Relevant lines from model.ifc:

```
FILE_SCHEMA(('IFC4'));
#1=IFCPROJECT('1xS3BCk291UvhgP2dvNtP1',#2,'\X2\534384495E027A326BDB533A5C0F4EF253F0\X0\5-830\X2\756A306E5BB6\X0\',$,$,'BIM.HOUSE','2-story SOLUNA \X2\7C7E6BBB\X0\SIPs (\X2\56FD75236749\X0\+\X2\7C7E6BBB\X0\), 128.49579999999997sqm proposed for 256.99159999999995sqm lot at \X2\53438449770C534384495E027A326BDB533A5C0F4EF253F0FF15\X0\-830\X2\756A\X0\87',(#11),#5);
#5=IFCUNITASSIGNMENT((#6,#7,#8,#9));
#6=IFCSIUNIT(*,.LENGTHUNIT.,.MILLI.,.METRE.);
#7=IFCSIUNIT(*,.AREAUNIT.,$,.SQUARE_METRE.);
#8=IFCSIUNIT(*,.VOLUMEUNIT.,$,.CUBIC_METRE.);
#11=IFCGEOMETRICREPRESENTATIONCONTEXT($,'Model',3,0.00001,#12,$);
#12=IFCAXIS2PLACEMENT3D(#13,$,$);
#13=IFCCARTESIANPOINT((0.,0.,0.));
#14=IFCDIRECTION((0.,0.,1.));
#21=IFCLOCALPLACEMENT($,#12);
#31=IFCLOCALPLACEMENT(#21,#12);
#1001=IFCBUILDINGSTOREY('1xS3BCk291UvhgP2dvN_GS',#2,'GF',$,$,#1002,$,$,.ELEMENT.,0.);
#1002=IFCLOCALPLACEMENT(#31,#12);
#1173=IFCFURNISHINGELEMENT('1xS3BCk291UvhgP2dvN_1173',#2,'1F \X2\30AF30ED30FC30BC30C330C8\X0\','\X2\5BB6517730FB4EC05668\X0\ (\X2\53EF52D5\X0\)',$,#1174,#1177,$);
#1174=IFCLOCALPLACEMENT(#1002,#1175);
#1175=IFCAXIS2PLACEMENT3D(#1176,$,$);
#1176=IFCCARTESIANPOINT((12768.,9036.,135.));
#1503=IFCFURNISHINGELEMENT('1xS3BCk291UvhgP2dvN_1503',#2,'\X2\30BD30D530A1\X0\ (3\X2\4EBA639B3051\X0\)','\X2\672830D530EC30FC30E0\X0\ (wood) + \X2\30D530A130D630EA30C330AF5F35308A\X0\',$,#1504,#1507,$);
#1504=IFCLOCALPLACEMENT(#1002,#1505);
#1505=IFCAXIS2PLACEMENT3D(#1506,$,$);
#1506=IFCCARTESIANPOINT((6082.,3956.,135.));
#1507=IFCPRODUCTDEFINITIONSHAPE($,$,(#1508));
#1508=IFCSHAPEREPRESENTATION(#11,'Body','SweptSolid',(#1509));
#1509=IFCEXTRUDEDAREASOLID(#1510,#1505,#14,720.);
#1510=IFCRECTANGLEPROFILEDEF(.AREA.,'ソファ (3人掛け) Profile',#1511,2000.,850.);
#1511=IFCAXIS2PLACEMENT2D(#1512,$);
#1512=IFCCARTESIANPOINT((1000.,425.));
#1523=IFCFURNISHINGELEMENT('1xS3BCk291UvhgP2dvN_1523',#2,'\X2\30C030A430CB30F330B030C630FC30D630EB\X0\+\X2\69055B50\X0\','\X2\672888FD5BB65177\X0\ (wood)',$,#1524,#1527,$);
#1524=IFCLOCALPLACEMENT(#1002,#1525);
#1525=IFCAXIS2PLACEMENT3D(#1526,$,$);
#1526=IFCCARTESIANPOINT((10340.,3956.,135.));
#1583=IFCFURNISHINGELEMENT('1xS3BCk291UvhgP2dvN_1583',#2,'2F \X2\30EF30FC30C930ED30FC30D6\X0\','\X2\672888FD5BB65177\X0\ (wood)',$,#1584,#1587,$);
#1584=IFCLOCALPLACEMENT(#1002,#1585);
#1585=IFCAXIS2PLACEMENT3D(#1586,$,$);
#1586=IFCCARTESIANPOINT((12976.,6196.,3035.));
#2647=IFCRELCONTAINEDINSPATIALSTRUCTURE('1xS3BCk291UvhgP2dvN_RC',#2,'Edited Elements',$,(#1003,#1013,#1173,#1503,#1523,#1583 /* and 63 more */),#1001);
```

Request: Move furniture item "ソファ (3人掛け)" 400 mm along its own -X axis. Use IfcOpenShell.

```python
import ifcopenshell
import ifcopenshell.api.geometry
import ifcopenshell.util.placement
import ifcopenshell.util.unit

model = ifcopenshell.open("model.ifc")
unit_scale = ifcopenshell.util.unit.calculate_unit_scale(model)

item = model.by_guid("1xS3BCk291UvhgP2dvN_1503")
matrix = ifcopenshell.util.placement.get_local_placement(item.ObjectPlacement)
matrix[:3, 3] -= matrix[:3, 0] * 0.4 / unit_scale
ifcopenshell.api.geometry.edit_object_placement(model, product=item, matrix=matrix, is_si=False)

print(ifcopenshell.util.placement.get_local_placement(item.ObjectPlacement).round(3) + 0.0)

model.write("model_rev.ifc")
```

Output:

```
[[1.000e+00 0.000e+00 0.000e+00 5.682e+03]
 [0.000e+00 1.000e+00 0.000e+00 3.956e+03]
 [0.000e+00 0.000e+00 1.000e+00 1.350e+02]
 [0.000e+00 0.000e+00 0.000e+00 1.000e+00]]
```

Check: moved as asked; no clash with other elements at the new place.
